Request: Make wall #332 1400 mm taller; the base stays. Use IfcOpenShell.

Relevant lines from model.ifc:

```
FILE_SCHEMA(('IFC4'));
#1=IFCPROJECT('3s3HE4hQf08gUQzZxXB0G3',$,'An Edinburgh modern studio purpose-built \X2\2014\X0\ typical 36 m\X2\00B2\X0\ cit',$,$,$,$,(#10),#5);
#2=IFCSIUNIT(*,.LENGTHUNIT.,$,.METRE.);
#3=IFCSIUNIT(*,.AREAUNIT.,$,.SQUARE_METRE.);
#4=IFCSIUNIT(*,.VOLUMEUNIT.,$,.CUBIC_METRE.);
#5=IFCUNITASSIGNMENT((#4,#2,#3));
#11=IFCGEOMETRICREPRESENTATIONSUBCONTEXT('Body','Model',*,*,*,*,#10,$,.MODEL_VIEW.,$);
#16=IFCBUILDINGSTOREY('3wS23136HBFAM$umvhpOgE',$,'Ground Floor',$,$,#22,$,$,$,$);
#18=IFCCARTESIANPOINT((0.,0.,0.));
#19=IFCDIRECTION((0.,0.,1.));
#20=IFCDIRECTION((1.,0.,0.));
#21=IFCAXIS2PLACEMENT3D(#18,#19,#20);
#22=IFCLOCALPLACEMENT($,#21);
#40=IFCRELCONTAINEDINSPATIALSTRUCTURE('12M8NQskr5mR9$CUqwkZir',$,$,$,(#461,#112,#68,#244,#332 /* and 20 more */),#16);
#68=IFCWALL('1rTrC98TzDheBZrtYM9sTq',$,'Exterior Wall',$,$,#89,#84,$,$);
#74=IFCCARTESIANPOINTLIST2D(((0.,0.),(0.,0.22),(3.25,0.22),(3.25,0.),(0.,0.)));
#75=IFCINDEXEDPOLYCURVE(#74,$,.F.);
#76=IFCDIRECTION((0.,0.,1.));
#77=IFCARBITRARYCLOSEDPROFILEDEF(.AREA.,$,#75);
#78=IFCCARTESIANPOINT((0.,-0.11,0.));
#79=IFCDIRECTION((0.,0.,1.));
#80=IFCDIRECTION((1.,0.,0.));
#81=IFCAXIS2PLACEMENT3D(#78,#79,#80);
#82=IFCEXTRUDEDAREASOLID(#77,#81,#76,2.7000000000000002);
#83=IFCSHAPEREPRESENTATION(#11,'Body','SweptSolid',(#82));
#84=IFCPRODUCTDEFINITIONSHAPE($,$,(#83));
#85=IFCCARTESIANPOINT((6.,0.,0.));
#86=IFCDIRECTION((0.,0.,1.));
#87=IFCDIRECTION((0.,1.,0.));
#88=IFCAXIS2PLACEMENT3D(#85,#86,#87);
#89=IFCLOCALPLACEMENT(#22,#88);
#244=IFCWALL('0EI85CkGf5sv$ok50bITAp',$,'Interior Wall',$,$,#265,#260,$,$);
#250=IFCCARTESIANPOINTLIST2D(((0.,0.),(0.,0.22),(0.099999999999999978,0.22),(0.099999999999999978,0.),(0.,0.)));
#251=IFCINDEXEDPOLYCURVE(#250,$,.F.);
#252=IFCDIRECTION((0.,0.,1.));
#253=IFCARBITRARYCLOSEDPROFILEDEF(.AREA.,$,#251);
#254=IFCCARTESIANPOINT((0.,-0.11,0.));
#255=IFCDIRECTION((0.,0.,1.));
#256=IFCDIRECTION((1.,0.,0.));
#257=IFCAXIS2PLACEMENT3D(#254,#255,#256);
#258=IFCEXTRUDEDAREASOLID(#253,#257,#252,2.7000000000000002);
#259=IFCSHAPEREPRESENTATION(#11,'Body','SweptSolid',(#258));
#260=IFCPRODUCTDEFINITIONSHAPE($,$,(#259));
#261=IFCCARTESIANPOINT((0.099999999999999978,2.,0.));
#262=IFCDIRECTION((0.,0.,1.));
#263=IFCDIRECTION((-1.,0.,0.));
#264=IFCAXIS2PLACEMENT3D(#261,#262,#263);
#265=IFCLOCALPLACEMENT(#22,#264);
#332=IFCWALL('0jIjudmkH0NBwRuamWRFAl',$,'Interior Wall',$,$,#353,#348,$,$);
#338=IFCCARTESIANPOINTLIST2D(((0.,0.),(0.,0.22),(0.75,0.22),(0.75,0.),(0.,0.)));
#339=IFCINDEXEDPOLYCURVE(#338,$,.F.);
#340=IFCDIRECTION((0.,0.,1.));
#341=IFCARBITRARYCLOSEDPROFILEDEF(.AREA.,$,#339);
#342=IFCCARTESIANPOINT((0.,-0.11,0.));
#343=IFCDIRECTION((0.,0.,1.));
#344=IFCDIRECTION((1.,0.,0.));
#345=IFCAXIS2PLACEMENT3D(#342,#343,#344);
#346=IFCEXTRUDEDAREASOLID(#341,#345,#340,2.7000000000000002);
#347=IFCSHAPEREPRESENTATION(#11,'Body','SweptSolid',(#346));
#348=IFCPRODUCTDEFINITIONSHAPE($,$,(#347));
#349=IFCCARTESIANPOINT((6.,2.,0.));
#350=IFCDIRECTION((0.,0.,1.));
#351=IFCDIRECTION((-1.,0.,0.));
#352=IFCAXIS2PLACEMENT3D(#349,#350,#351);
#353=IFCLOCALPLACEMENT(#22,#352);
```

```python
import ifcopenshell
import ifcopenshell.geom
import ifcopenshell.util.representation
import ifcopenshell.util.shape
import ifcopenshell.util.unit

model = ifcopenshell.open("model.ifc")
unit_scale = ifcopenshell.util.unit.calculate_unit_scale(model)
settings = ifcopenshell.geom.settings()


def volume(element):
    """Net volume in cubic metres, openings subtracted."""
    shape = ifcopenshell.geom.create_shape(settings, element)
    return ifcopenshell.util.shape.get_volume(shape.geometry)


wall = model.by_id(332)
before = volume(wall)

body = ifcopenshell.util.representation.get_representation(wall, "Model", "Body")
solid = body.Items[0]
old_height = solid.Depth
solid.Depth += 1.4 / unit_scale
after = volume(wall)

print(f"height {old_height:g} -> {solid.Depth:g}, volume {before:.3f} -> {after:.3f} m3")

model.write("model_updated.ifc")
```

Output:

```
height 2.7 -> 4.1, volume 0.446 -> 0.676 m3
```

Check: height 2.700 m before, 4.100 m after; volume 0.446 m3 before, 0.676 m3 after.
